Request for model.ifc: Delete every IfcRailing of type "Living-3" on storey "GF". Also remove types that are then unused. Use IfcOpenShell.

First a look at what the model holds.

```python
import ifcopenshell
import ifcopenshell.util.element

model = ifcopenshell.open("model.ifc")
print(model.schema)
storey = next(s for s in model.by_type("IfcBuildingStorey") if s.Name == "GF")
railings = [e for e in ifcopenshell.util.element.get_decomposition(storey) if e.is_a("IfcRailing")]
seen = {}
for e in railings:
    element_type = ifcopenshell.util.element.get_type(e)
    name = element_type.Name if element_type not in (None, e) else None
    seen[name] = seen.get(name, 0) + 1
for name, count in sorted(seen.items(), key=str):
    print(count, "x", name)
```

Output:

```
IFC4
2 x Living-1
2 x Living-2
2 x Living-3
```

```python
import ifcopenshell
import ifcopenshell.api.root
import ifcopenshell.util.element

model = ifcopenshell.open("model.ifc")

storey = next(s for s in model.by_type("IfcBuildingStorey") if s.Name == "GF")
railings = [e for e in ifcopenshell.util.element.get_decomposition(storey) if e.is_a("IfcRailing")]
targets = [e for e in railings if (t := ifcopenshell.util.element.get_type(e)) not in (None, e) and t.Name == "Living-3"]
types = {ifcopenshell.util.element.get_type(e) for e in targets} - {None, *targets}

for e in targets:
    ifcopenshell.api.root.remove_product(model, product=e)
print(len(targets), "removed")

unused = [t for t in types if not ifcopenshell.util.element.get_types(t)]
for t in unused:
    ifcopenshell.api.root.remove_product(model, product=t)
print(len(unused), "unused types removed")

model.write("model_v2.ifc")
```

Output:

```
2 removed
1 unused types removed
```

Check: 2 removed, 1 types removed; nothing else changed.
